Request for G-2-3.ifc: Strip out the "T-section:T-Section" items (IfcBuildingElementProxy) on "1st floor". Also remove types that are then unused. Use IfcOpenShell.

First a look at what the model holds.

```python
import ifcopenshell
import ifcopenshell.util.element

model = ifcopenshell.open("G-2-3.ifc")
print(model.schema)
storey = next(s for s in model.by_type("IfcBuildingStorey") if s.Name == "1st floor")
proxies = [e for e in ifcopenshell.util.element.get_decomposition(storey) if e.is_a("IfcBuildingElementProxy")]
seen = {}
for e in proxies:
    element_type = ifcopenshell.util.element.get_type(e)
    name = element_type.Name if element_type not in (None, e) else None
    seen[name] = seen.get(name, 0) + 1
for name, count in sorted(seen.items(), key=str):
    print(count, "x", name)
```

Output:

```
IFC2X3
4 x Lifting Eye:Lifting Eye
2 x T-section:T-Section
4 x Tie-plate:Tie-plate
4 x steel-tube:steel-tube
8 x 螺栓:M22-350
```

```python
import ifcopenshell
import ifcopenshell.api.root
import ifcopenshell.util.element

model = ifcopenshell.open("G-2-3.ifc")

storey = next(s for s in model.by_type("IfcBuildingStorey") if s.Name == "1st floor")
proxies = [e for e in ifcopenshell.util.element.get_decomposition(storey) if e.is_a("IfcBuildingElementProxy")]
targets = [e for e in proxies if (t := ifcopenshell.util.element.get_type(e)) not in (None, e) and t.Name == "T-section:T-Section"]
types = {ifcopenshell.util.element.get_type(e) for e in targets} - {None, *targets}

for e in targets:
    ifcopenshell.api.root.remove_product(model, product=e)
print(len(targets), "removed")

unused = [t for t in types if not ifcopenshell.util.element.get_types(t)]
for t in unused:
    ifcopenshell.api.root.remove_product(model, product=t)
print(len(unused), "unused types removed")

model.write("G-2-3_edited.ifc")
```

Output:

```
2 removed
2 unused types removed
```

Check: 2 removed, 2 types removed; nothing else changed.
